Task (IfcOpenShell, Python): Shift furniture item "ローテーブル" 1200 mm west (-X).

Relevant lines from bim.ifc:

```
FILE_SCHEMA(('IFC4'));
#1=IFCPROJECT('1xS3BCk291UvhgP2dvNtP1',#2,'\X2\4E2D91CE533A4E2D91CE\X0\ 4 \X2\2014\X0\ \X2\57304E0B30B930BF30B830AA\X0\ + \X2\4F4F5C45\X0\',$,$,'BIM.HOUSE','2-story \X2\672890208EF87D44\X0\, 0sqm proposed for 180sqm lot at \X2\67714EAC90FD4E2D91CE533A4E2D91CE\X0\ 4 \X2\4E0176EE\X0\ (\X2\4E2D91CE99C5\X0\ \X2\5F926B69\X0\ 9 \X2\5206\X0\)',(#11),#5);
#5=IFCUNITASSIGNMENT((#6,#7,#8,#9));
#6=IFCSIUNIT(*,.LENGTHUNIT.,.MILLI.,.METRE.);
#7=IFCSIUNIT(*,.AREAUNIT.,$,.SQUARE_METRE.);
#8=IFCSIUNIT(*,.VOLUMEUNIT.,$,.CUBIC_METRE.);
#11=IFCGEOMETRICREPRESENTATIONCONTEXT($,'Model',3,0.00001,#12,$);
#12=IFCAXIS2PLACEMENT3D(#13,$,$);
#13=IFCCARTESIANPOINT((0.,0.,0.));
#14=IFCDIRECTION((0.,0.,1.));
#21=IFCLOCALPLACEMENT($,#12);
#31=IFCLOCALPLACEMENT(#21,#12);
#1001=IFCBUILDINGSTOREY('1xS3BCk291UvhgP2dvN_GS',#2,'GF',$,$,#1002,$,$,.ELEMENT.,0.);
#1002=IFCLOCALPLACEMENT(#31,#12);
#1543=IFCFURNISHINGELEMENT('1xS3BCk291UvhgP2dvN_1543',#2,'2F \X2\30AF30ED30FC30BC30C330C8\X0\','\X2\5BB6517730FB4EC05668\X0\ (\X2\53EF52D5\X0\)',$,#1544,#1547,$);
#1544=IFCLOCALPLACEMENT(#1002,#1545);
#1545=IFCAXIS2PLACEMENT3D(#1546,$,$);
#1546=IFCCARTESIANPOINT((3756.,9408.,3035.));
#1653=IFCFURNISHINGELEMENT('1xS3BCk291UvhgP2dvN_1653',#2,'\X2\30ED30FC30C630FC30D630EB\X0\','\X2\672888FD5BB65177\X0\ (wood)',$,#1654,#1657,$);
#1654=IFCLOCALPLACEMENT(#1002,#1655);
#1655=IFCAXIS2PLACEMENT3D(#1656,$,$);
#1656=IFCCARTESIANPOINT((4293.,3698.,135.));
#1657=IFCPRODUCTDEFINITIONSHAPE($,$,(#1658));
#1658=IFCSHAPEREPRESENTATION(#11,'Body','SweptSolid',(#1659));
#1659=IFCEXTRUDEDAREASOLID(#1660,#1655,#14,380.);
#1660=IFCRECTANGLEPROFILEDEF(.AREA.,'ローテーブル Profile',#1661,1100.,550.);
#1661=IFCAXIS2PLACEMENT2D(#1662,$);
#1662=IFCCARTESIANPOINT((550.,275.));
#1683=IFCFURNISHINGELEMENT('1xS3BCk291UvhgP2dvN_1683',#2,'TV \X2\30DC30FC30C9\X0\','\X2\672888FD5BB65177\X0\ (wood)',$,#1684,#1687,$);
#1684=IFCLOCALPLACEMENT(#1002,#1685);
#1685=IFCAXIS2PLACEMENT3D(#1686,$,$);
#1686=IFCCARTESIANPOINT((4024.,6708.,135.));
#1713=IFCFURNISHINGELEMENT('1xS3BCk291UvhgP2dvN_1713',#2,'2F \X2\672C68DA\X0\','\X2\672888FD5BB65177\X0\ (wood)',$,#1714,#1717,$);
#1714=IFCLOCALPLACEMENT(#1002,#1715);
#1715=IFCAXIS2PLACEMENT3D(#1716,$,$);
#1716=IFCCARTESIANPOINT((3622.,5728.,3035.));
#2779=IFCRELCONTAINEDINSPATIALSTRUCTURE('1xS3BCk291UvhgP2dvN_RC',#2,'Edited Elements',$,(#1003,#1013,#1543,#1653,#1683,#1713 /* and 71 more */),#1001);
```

```python
import ifcopenshell
import ifcopenshell.api.geometry
import ifcopenshell.util.placement

model = ifcopenshell.open("bim.ifc")

item = model.by_id(1653)
matrix = ifcopenshell.util.placement.get_local_placement(item.ObjectPlacement)
matrix[0, 3] -= 1200.0
ifcopenshell.api.geometry.edit_object_placement(model, product=item, matrix=matrix, is_si=False)

print(ifcopenshell.util.placement.get_local_placement(item.ObjectPlacement).round(3) + 0.0)

model.write("bim-out.ifc")
```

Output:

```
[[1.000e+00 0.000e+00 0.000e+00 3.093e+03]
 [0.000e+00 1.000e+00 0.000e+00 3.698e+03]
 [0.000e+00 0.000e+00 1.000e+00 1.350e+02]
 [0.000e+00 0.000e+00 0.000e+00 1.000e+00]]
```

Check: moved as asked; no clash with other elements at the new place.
